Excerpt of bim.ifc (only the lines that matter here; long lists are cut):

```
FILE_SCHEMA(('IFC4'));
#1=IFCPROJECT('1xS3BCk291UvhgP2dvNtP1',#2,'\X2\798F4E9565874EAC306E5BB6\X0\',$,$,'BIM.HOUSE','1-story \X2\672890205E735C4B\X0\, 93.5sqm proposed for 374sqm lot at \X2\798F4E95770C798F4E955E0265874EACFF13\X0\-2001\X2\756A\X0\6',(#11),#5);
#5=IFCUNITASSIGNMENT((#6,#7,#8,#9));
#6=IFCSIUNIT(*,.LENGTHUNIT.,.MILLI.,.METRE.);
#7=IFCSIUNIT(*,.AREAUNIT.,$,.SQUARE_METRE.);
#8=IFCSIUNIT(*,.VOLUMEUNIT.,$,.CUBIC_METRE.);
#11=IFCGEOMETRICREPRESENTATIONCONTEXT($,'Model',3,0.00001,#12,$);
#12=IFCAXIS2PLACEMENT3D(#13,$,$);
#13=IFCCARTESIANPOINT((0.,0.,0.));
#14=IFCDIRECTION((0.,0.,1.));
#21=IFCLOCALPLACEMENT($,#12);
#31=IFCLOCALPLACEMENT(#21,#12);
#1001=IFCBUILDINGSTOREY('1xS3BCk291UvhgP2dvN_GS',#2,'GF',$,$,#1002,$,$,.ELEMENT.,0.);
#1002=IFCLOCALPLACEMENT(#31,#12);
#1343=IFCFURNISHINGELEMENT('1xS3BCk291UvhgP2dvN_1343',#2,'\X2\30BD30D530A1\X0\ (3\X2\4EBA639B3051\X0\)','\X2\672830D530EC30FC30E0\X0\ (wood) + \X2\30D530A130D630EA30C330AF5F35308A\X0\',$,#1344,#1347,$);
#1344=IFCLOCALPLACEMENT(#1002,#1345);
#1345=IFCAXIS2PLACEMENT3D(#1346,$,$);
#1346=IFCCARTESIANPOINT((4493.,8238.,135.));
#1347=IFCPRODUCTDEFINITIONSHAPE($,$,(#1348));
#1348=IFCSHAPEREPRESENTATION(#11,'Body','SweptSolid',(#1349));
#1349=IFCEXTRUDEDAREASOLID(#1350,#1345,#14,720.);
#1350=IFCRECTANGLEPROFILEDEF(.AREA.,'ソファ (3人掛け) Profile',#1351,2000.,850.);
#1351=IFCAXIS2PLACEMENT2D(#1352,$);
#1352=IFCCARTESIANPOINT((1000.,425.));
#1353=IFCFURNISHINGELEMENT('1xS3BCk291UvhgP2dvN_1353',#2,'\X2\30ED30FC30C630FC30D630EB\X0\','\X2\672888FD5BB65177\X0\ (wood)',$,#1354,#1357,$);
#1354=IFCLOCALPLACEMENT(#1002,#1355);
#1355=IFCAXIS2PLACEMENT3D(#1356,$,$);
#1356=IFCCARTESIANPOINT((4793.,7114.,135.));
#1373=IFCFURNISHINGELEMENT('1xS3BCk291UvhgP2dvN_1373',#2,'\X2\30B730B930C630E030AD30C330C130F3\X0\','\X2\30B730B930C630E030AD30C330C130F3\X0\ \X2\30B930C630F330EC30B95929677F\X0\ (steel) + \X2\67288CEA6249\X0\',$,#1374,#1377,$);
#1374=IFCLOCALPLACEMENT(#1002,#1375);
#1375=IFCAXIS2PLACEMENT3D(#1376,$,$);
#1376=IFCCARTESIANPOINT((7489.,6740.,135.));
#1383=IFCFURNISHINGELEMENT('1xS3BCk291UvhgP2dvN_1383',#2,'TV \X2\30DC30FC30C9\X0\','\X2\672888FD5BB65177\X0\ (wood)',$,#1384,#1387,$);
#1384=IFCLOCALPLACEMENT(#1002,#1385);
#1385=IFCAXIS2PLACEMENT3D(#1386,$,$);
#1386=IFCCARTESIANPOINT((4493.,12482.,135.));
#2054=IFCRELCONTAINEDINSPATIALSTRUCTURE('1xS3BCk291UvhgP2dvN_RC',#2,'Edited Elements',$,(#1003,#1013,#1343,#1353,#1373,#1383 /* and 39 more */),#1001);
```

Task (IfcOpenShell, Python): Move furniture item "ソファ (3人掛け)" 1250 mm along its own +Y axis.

```python
import ifcopenshell
import ifcopenshell.api.geometry
import ifcopenshell.util.placement
import ifcopenshell.util.unit

model = ifcopenshell.open("bim.ifc")
unit_scale = ifcopenshell.util.unit.calculate_unit_scale(model)

item = model.by_guid("1xS3BCk291UvhgP2dvN_1343")
matrix = ifcopenshell.util.placement.get_local_placement(item.ObjectPlacement)
matrix[:3, 3] += matrix[:3, 1] * 1.25 / unit_scale
ifcopenshell.api.geometry.edit_object_placement(model, product=item, matrix=matrix, is_si=False)

print(ifcopenshell.util.placement.get_local_placement(item.ObjectPlacement).round(3) + 0.0)

model.write("bim_rev.ifc")
```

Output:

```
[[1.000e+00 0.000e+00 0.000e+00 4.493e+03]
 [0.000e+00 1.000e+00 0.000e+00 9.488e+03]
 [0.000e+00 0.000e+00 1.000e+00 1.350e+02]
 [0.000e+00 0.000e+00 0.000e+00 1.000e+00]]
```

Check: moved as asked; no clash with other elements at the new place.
